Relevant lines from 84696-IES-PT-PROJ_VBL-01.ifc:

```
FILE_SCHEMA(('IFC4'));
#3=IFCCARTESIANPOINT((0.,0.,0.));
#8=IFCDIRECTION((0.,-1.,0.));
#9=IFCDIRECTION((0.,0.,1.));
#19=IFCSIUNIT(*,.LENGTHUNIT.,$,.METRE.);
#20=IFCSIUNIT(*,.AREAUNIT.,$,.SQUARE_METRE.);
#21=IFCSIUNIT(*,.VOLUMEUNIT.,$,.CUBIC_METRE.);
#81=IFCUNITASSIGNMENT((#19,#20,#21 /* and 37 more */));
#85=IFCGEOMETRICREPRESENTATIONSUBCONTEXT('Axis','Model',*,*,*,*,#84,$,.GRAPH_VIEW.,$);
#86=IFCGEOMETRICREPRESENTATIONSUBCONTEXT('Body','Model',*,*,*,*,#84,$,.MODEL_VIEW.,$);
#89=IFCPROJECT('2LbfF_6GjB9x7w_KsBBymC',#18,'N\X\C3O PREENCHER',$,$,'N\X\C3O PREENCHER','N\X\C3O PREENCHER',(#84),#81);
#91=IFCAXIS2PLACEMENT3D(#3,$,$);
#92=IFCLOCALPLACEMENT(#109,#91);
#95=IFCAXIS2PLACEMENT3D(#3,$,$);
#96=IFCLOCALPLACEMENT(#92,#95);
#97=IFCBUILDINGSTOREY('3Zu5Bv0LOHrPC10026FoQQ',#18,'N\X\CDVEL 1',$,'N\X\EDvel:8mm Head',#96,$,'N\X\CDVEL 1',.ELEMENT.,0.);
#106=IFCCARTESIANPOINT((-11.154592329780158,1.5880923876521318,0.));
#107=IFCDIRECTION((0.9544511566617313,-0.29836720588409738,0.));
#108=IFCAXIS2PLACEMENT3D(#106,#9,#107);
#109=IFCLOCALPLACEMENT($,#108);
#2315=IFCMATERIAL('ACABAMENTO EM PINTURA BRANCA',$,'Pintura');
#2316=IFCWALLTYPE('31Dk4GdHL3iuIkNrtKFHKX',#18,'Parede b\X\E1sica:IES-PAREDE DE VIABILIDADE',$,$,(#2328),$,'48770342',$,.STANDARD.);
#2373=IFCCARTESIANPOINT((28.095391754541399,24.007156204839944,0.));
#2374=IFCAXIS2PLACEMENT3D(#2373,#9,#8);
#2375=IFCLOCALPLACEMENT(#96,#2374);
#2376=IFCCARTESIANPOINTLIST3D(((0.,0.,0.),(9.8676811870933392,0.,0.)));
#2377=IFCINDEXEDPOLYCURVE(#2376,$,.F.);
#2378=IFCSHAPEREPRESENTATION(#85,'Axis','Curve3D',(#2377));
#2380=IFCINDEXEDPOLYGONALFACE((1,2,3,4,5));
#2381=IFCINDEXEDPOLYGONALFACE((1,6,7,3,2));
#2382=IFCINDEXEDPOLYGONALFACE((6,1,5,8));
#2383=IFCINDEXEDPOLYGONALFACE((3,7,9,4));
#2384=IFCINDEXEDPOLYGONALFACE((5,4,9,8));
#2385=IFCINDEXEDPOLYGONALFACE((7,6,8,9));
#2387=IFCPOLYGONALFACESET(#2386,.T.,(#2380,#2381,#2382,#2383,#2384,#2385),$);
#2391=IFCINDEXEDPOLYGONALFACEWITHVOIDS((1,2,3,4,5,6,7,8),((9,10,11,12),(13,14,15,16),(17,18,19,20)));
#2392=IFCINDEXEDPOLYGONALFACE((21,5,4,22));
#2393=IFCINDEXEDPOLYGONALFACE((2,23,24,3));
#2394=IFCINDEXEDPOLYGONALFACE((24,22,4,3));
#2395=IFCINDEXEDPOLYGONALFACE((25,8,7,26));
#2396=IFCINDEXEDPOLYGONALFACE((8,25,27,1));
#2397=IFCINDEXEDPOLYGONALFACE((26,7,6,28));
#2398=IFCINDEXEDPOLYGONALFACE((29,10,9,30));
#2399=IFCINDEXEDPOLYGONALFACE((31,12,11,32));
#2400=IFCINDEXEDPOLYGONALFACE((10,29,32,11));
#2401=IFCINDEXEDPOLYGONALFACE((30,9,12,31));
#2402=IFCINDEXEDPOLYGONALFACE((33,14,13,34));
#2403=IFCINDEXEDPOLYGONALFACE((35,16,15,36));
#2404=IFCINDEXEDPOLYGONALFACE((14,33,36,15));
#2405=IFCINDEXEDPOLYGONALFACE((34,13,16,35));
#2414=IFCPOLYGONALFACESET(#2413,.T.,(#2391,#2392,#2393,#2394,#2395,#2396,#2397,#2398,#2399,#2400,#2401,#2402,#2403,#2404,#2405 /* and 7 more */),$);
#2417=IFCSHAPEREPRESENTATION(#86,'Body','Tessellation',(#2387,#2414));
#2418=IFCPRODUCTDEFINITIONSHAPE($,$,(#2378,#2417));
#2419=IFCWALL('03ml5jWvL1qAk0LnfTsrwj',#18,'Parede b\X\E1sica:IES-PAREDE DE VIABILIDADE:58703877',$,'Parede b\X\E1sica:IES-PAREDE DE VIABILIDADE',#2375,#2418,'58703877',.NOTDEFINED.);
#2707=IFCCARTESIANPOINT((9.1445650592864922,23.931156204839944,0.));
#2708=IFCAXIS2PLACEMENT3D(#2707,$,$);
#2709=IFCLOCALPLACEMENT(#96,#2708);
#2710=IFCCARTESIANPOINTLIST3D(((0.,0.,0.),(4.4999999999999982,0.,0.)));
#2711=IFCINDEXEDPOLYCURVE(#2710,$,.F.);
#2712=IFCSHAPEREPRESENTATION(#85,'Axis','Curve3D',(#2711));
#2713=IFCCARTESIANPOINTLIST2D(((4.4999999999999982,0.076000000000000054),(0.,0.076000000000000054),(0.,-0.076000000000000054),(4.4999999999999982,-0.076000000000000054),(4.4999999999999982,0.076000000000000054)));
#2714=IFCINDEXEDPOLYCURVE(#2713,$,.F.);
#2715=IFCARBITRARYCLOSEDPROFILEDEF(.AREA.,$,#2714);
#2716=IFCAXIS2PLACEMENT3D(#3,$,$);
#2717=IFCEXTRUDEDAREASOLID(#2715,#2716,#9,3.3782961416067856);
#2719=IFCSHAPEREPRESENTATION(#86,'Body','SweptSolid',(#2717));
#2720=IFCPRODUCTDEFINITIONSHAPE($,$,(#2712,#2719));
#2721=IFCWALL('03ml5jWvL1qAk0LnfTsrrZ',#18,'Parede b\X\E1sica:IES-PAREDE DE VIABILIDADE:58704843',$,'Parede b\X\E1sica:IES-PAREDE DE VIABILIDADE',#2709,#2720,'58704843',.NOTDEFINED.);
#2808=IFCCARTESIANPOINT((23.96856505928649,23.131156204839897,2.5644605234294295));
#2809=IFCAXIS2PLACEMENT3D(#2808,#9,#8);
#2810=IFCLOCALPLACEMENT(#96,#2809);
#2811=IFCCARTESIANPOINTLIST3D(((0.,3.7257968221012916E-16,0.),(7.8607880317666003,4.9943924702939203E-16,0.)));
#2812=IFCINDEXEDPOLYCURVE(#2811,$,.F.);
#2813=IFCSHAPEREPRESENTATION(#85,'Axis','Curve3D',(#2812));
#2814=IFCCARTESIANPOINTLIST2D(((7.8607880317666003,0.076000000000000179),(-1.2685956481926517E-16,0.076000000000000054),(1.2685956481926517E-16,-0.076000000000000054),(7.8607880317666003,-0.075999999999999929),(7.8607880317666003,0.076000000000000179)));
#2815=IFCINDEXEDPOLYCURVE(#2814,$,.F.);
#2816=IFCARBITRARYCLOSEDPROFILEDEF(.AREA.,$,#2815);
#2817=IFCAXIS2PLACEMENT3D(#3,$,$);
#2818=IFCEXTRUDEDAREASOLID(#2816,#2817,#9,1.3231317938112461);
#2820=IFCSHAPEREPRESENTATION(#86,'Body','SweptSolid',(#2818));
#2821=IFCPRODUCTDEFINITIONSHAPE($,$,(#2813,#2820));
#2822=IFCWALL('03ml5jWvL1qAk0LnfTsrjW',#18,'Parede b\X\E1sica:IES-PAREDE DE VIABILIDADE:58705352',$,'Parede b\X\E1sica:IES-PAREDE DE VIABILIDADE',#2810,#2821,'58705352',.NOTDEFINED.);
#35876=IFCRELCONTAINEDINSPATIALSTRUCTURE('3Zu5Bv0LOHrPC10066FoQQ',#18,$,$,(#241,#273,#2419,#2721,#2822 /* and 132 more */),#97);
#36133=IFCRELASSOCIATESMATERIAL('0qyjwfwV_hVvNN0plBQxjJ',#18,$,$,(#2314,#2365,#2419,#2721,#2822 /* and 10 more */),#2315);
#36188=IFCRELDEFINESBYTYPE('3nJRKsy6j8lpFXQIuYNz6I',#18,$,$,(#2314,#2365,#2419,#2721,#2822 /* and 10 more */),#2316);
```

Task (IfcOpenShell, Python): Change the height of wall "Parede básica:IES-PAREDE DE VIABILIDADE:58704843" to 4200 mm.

```python
import ifcopenshell
import ifcopenshell.geom
import ifcopenshell.util.representation
import ifcopenshell.util.shape

model = ifcopenshell.open("84696-IES-PT-PROJ_VBL-01.ifc")
settings = ifcopenshell.geom.settings()


def volume(element):
    """Net volume in cubic metres, openings subtracted."""
    shape = ifcopenshell.geom.create_shape(settings, element)
    return ifcopenshell.util.shape.get_volume(shape.geometry)


wall = model.by_guid("03ml5jWvL1qAk0LnfTsrrZ")
before = volume(wall)

body = ifcopenshell.util.representation.get_representation(wall, "Model", "Body")
solid = body.Items[0]
old_height = solid.Depth
solid.Depth = 4.2
after = volume(wall)

print(f"height {old_height:g} -> {solid.Depth:g}, volume {before:.3f} -> {after:.3f} m3")

model.write("84696-IES-PT-PROJ_VBL-01_edited.ifc")
```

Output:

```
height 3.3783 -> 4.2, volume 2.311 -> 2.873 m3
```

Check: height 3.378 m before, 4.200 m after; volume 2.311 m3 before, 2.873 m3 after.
